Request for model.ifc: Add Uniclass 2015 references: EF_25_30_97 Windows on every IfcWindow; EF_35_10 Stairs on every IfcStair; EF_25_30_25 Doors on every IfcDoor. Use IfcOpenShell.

First a look at what the model holds.

```python
import ifcopenshell

model = ifcopenshell.open("model.ifc")
print(model.schema)
print("classifications:", [c.Name for c in model.by_type("IfcClassification")])
for ifc_class in ("IfcDoor", "IfcRoof", "IfcStair", "IfcWall", "IfcWindow"):
    print(ifc_class, len(model.by_type(ifc_class)))
```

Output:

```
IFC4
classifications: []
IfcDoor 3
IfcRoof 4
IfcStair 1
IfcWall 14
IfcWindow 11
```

```python
import ifcopenshell
import ifcopenshell.api.classification

model = ifcopenshell.open("model.ifc")

system = ifcopenshell.api.classification.add_classification(model, classification="Uniclass 2015")

codes = {
    "IfcWindow": ("EF_25_30_97", "Windows"),
    "IfcStair": ("EF_35_10", "Stairs"),
    "IfcDoor": ("EF_25_30_25", "Doors"),
}
for ifc_class, (code, name) in codes.items():
    products = model.by_type(ifc_class)
    ifcopenshell.api.classification.add_reference(
        model, products=products, classification=system, identification=code, name=name
    )
    print(code, len(products))

model.write("model-out.ifc")
```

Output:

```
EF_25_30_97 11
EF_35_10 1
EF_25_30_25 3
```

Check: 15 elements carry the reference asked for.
